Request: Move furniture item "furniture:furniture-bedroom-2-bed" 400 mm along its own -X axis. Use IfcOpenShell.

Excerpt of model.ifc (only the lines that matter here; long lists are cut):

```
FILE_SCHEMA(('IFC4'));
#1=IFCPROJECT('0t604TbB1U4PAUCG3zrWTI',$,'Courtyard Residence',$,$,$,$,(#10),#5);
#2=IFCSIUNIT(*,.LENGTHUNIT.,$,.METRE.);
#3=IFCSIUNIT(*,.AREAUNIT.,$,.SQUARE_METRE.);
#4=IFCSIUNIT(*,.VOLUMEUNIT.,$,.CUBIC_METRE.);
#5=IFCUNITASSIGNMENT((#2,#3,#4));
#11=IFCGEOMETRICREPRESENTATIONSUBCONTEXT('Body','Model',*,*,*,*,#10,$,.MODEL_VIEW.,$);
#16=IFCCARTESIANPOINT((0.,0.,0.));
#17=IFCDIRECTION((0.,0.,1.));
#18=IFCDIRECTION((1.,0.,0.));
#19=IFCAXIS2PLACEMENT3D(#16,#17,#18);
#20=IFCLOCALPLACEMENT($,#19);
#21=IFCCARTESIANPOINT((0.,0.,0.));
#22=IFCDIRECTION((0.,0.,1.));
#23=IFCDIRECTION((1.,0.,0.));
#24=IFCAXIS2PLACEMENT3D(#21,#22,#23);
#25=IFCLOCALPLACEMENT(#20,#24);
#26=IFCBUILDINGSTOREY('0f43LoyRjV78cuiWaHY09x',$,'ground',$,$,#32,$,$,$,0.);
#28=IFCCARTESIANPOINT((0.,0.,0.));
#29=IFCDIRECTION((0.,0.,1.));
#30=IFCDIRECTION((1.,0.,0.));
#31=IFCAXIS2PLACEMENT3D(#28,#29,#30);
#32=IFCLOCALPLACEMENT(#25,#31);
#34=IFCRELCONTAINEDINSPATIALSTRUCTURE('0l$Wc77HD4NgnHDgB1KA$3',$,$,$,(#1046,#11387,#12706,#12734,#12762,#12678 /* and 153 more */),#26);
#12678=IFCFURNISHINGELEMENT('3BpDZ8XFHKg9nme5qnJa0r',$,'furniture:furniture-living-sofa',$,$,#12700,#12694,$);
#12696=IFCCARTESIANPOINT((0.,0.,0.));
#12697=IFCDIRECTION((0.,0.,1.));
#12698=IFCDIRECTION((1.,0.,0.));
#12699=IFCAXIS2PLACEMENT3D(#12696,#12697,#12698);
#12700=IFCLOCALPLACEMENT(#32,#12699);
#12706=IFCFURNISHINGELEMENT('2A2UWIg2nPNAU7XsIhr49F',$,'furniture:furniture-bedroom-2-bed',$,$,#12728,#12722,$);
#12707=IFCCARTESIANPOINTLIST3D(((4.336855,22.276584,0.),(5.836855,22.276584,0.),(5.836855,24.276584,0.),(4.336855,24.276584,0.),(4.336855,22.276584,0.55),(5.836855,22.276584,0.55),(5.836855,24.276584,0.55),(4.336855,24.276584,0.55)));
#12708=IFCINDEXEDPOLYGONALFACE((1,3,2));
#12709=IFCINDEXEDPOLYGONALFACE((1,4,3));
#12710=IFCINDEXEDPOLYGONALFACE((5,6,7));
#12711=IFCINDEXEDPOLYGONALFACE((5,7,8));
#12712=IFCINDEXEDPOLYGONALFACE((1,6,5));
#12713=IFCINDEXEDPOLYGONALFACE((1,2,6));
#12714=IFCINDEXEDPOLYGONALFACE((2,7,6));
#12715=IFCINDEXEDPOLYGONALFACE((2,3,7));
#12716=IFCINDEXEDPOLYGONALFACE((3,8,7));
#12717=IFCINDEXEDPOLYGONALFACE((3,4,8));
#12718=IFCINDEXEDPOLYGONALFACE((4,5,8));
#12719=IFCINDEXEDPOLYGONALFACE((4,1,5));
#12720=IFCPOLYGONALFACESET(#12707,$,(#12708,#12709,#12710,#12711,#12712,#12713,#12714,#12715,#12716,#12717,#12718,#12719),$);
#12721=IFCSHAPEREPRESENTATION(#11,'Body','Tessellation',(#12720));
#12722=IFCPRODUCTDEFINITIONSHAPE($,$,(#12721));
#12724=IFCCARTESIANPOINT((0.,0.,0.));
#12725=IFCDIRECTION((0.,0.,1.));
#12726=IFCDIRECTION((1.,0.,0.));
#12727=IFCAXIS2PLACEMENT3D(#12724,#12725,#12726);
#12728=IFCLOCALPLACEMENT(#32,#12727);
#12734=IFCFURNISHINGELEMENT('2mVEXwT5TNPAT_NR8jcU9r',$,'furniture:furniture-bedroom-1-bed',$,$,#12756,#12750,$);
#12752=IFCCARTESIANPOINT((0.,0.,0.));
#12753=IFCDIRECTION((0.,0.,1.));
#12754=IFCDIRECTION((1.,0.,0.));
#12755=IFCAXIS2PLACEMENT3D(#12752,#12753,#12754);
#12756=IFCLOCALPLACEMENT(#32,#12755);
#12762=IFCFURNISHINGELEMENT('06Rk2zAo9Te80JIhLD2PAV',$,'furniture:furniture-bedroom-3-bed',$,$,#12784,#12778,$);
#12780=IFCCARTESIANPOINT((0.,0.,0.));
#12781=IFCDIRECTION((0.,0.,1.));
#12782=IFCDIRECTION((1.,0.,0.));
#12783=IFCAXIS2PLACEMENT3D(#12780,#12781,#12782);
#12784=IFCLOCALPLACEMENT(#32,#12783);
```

```python
import ifcopenshell
import ifcopenshell.api.geometry
import ifcopenshell.util.placement
import ifcopenshell.util.unit

model = ifcopenshell.open("model.ifc")
unit_scale = ifcopenshell.util.unit.calculate_unit_scale(model)

item = model.by_id(12706)
matrix = ifcopenshell.util.placement.get_local_placement(item.ObjectPlacement)
matrix[:3, 3] -= matrix[:3, 0] * 0.4 / unit_scale
ifcopenshell.api.geometry.edit_object_placement(model, product=item, matrix=matrix, is_si=False)

print(ifcopenshell.util.placement.get_local_placement(item.ObjectPlacement).round(3) + 0.0)

model.write("model_edited.ifc")
```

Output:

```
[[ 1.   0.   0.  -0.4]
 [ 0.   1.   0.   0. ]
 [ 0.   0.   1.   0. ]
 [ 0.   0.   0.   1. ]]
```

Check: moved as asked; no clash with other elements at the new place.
